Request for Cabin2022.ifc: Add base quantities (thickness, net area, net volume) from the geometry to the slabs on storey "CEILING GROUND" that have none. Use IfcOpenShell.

First a look at what the model holds.

```python
import ifcopenshell
import ifcopenshell.util.element
import ifcopenshell.util.unit

model = ifcopenshell.open("Cabin2022.ifc")
print(model.schema)
for unit_type in ("LENGTHUNIT", "AREAUNIT", "VOLUMEUNIT"):
    print(unit_type, ifcopenshell.util.unit.calculate_unit_scale(model, unit_type))
storey = next(s for s in model.by_type("IfcBuildingStorey") if s.Name == "CEILING GROUND")
slabs = [e for e in ifcopenshell.util.element.get_decomposition(storey) if e.is_a("IfcSlab")]
for e in sorted(slabs, key=lambda e: e.id()):
    print(e.id(), e.is_a(), e.Name, list(ifcopenshell.util.element.get_psets(e, qtos_only=True)), sep=" | ")
```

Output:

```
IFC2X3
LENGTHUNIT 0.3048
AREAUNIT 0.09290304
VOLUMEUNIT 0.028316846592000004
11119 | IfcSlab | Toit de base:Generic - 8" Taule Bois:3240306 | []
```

```python
import ifcopenshell
import ifcopenshell.api.pset
import ifcopenshell.geom
import ifcopenshell.util.element
import ifcopenshell.util.shape
import ifcopenshell.util.unit

model = ifcopenshell.open("Cabin2022.ifc")
unit_scale = ifcopenshell.util.unit.calculate_unit_scale(model)
area_scale = ifcopenshell.util.unit.calculate_unit_scale(model, "AREAUNIT")
volume_scale = ifcopenshell.util.unit.calculate_unit_scale(model, "VOLUMEUNIT")
settings = ifcopenshell.geom.settings()

storey = next(s for s in model.by_type("IfcBuildingStorey") if s.Name == "CEILING GROUND")
slabs = [e for e in ifcopenshell.util.element.get_decomposition(storey) if e.is_a("IfcSlab")]

for e in sorted(slabs, key=lambda e: e.id()):
    if ifcopenshell.util.element.get_psets(e, qtos_only=True, should_inherit=False):
        continue
    # Geometry comes back in metres, in the element's own axes.
    shape = ifcopenshell.geom.create_shape(settings, e)
    values = {
        "Width": ifcopenshell.util.shape.get_z(shape.geometry) / unit_scale,
        "NetArea": ifcopenshell.util.shape.get_footprint_area(shape.geometry) / area_scale,
        "NetVolume": ifcopenshell.util.shape.get_volume(shape.geometry) / volume_scale,
    }
    qto = ifcopenshell.api.pset.add_qto(model, product=e, name="BaseQuantities")
    ifcopenshell.api.pset.edit_qto(model, qto=qto, properties=values)
    print(e.id(), {k: round(v, 3) for k, v in values.items()})

model.write("Cabin2022_v2.ifc")
```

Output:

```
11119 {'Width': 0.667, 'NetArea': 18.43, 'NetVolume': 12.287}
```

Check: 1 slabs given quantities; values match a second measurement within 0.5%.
